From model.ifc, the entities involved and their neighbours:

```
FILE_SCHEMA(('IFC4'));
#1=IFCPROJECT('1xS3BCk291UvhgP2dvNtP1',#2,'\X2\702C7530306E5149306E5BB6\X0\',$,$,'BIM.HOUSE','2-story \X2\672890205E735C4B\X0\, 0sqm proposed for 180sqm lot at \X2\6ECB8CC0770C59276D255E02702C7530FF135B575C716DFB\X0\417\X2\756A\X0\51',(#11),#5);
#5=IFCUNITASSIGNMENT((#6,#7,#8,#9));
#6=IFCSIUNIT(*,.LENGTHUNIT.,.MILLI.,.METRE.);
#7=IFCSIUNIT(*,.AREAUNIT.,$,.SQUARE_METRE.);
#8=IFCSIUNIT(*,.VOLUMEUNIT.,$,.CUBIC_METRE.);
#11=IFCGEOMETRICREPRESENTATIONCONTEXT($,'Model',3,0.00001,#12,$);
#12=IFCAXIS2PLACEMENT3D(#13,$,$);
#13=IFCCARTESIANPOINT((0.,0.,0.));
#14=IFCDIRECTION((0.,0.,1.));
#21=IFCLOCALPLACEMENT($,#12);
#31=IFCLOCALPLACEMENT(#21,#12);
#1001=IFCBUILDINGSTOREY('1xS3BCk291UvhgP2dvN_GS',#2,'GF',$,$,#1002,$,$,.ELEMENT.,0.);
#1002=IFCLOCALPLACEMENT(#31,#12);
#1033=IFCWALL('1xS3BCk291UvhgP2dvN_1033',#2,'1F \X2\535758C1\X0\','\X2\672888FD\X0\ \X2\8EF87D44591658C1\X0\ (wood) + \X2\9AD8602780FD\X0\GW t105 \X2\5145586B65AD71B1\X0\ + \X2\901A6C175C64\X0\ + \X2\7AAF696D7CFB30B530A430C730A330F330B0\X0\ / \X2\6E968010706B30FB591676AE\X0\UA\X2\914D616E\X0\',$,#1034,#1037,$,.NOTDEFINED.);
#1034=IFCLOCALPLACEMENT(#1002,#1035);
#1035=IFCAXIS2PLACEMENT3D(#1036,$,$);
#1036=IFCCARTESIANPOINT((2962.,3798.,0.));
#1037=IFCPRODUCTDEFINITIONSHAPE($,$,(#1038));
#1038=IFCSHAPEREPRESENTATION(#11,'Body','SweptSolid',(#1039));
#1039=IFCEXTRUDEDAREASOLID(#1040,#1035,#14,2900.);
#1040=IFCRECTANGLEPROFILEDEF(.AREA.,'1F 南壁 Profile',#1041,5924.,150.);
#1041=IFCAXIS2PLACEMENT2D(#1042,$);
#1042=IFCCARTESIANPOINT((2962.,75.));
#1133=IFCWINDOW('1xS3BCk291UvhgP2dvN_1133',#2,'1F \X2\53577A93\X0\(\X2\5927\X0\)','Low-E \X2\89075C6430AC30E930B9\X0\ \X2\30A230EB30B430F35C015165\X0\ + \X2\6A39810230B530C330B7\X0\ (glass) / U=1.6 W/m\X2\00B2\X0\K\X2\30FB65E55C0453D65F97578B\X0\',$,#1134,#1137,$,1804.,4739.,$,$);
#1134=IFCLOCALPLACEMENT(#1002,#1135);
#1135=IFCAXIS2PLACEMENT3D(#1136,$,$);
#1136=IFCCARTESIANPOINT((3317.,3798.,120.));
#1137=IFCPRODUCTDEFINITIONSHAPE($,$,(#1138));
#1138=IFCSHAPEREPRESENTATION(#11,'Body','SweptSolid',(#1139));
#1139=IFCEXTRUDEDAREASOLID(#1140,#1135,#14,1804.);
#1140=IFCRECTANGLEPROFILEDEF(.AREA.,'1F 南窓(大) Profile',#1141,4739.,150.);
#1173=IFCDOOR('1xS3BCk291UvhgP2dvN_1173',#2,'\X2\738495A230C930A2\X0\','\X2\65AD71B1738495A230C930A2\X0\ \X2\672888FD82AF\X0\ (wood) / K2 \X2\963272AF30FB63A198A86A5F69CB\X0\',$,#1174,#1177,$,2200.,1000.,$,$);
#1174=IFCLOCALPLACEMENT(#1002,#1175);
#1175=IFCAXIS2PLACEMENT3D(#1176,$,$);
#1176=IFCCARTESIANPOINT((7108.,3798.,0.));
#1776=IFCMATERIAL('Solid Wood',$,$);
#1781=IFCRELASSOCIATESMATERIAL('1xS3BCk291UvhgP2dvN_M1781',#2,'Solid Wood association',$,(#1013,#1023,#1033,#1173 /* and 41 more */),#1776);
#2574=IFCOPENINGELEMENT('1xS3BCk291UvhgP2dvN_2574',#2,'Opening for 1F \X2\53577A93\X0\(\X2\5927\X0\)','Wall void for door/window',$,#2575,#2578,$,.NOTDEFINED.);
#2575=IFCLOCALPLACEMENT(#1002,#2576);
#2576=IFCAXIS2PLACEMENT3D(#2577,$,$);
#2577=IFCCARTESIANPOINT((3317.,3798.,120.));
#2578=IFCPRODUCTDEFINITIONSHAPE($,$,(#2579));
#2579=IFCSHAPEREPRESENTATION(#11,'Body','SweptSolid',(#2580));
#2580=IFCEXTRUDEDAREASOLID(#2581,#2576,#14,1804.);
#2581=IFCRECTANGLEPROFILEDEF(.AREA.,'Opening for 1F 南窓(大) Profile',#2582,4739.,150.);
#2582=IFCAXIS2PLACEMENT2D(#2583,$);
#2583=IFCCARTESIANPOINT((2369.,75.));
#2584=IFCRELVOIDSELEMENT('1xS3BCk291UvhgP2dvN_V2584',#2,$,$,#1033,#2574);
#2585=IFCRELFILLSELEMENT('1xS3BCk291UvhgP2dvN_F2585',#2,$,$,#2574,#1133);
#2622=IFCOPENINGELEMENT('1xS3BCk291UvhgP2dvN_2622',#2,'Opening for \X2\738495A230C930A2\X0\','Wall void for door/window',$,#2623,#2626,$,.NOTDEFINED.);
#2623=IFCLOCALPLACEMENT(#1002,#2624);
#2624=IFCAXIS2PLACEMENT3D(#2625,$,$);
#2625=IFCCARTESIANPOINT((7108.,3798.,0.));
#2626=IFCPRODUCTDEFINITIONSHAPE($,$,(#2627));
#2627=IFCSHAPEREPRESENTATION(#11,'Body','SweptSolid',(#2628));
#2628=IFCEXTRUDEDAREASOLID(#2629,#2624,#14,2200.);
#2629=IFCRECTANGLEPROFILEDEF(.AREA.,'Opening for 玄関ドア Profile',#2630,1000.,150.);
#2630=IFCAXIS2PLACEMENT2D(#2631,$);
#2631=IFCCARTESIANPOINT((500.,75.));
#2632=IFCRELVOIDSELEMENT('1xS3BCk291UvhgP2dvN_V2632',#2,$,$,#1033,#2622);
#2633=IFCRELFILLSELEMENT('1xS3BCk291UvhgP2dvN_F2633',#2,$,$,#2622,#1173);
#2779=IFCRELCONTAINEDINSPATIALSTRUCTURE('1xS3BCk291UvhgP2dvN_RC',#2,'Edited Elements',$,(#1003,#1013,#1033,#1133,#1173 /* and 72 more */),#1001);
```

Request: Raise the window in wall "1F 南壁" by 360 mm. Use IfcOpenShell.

```python
import numpy as np
import ifcopenshell
import ifcopenshell.api.geometry
import ifcopenshell.util.placement
import ifcopenshell.util.unit

model = ifcopenshell.open("model.ifc")
unit_scale = ifcopenshell.util.unit.calculate_unit_scale(model)

window = model.by_guid("1xS3BCk291UvhgP2dvN_1133")
opening = window.FillsVoids[0].RelatingOpeningElement
dz = 0.36 / unit_scale

shift = np.array([0.0, 0.0, dz])
# The window is not placed relative to its opening, so move both.
for product in (opening, window):
    matrix = ifcopenshell.util.placement.get_local_placement(product.ObjectPlacement)
    matrix[:3, 3] += shift
    ifcopenshell.api.geometry.edit_object_placement(model, product=product, matrix=matrix, is_si=False)

print(f"moved by {dz * unit_scale:+.3f} m")

model.write("model_v2.ifc")
```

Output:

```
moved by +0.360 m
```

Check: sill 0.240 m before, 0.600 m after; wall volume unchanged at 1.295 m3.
